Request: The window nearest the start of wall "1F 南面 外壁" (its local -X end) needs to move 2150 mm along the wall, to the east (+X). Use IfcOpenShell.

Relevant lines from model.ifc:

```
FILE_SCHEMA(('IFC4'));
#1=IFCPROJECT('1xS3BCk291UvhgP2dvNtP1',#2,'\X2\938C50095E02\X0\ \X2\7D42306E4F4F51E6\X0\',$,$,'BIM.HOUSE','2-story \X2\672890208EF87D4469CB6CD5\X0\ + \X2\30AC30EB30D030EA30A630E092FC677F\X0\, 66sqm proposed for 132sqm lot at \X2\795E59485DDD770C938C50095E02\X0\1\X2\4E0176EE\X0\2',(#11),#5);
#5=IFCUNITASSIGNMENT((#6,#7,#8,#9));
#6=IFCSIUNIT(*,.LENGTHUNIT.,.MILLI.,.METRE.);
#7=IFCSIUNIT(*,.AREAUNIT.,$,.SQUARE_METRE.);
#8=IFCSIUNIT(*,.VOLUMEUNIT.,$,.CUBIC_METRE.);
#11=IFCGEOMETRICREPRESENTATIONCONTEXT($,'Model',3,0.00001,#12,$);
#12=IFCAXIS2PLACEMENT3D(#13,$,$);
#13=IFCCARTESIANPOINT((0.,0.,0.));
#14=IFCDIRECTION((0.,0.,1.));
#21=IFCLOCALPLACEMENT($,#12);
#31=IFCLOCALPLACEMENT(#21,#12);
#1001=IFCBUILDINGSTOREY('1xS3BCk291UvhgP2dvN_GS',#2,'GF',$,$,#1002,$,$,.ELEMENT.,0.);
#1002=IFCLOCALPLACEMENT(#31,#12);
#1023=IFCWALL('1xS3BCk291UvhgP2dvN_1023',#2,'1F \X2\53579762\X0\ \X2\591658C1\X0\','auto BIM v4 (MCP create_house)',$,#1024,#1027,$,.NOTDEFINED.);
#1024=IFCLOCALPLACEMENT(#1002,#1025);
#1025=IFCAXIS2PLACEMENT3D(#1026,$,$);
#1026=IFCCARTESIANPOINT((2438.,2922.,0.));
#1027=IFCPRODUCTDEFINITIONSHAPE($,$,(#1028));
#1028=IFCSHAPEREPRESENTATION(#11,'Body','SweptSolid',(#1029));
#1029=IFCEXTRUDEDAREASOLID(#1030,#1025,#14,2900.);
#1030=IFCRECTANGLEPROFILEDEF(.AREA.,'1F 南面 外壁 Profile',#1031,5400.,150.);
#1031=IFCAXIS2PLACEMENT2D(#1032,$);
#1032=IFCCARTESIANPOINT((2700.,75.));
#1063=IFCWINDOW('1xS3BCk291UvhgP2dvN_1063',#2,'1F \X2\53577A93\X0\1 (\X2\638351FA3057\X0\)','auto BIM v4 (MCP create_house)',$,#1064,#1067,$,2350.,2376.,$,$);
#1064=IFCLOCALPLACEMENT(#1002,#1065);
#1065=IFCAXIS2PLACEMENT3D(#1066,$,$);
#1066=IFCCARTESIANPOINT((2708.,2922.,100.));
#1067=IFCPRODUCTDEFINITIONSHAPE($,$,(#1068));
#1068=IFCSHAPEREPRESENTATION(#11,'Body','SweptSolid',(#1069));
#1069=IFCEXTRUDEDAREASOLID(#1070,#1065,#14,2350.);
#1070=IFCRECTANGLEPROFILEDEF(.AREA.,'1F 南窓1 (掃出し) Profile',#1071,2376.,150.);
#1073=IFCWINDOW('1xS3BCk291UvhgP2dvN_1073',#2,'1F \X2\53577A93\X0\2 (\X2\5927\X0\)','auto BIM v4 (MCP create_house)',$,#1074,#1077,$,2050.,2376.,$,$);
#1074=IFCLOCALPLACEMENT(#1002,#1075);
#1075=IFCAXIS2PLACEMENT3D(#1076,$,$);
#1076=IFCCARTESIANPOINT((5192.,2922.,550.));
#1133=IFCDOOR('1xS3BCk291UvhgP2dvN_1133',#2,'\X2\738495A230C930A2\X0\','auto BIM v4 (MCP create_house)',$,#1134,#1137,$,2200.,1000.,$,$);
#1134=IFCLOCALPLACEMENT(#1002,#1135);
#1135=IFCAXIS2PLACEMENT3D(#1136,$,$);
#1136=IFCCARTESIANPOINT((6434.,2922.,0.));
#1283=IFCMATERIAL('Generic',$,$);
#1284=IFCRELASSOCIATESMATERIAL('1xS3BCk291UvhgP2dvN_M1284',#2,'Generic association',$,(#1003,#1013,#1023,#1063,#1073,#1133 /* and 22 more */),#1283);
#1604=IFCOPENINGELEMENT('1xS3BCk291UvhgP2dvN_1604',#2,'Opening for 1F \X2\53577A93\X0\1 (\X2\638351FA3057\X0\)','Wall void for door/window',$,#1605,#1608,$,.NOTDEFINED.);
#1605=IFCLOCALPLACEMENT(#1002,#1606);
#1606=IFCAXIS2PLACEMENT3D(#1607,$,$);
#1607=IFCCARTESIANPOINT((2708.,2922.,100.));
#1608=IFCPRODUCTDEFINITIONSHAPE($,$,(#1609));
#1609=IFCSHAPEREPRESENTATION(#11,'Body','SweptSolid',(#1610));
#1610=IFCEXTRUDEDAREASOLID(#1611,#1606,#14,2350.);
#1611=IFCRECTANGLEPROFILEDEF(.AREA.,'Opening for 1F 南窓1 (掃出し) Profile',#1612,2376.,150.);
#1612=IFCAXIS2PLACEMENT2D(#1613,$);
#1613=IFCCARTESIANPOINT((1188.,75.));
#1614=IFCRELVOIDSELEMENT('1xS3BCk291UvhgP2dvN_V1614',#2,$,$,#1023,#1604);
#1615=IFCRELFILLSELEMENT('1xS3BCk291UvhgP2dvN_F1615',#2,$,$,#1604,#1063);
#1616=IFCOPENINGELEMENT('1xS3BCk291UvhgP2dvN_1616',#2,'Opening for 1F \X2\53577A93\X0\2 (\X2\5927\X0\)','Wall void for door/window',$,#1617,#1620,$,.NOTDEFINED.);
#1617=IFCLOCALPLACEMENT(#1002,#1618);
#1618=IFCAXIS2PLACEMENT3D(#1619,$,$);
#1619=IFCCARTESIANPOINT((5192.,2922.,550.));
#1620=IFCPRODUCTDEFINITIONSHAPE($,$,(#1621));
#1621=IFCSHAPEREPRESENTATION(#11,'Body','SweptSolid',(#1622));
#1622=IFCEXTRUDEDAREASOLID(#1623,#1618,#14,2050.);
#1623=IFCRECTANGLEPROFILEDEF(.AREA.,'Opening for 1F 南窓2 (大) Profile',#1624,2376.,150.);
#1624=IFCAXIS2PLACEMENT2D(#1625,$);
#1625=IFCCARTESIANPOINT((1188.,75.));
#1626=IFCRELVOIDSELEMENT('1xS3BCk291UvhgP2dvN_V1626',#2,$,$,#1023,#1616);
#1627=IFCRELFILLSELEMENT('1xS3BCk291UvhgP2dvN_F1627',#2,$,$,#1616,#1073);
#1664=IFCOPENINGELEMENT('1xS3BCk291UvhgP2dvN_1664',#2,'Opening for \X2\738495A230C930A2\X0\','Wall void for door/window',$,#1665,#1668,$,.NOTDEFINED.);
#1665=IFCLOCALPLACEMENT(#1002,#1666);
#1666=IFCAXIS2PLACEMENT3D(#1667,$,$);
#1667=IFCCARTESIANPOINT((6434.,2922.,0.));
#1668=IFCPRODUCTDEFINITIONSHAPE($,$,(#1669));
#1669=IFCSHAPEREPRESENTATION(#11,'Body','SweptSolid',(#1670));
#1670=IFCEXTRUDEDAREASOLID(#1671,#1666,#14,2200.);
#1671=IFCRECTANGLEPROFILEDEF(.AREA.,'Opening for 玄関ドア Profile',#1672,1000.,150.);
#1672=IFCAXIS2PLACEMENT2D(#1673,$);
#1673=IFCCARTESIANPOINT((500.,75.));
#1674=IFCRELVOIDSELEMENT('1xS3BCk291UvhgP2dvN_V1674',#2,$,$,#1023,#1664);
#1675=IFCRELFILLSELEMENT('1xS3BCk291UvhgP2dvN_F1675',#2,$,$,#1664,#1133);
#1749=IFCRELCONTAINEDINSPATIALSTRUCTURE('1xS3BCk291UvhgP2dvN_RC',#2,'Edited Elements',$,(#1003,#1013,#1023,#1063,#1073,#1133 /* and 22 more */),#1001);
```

```python
import ifcopenshell
import ifcopenshell.api.geometry
import ifcopenshell.util.placement
import ifcopenshell.util.unit

model = ifcopenshell.open("model.ifc")
unit_scale = ifcopenshell.util.unit.calculate_unit_scale(model)

window = model.by_id(1063)
opening = window.FillsVoids[0].RelatingOpeningElement
wall = opening.VoidsElements[0].RelatingBuildingElement

wall_matrix = ifcopenshell.util.placement.get_local_placement(wall.ObjectPlacement)
shift = wall_matrix[:3, 0] * 2.15 / unit_scale
before = ifcopenshell.util.placement.get_local_placement(window.ObjectPlacement)[:3, 3].copy()

# The window is not placed relative to its opening, so move both.
for product in (opening, window):
    matrix = ifcopenshell.util.placement.get_local_placement(product.ObjectPlacement)
    matrix[:3, 3] += shift
    ifcopenshell.api.geometry.edit_object_placement(model, product=product, matrix=matrix, is_si=False)

after = ifcopenshell.util.placement.get_local_placement(window.ObjectPlacement)[:3, 3]
print("window moved by", (after - before).round(3) + 0.0)

model.write("model_edited.ifc")
```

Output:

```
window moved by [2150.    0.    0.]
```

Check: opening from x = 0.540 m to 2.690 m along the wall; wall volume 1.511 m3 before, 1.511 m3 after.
